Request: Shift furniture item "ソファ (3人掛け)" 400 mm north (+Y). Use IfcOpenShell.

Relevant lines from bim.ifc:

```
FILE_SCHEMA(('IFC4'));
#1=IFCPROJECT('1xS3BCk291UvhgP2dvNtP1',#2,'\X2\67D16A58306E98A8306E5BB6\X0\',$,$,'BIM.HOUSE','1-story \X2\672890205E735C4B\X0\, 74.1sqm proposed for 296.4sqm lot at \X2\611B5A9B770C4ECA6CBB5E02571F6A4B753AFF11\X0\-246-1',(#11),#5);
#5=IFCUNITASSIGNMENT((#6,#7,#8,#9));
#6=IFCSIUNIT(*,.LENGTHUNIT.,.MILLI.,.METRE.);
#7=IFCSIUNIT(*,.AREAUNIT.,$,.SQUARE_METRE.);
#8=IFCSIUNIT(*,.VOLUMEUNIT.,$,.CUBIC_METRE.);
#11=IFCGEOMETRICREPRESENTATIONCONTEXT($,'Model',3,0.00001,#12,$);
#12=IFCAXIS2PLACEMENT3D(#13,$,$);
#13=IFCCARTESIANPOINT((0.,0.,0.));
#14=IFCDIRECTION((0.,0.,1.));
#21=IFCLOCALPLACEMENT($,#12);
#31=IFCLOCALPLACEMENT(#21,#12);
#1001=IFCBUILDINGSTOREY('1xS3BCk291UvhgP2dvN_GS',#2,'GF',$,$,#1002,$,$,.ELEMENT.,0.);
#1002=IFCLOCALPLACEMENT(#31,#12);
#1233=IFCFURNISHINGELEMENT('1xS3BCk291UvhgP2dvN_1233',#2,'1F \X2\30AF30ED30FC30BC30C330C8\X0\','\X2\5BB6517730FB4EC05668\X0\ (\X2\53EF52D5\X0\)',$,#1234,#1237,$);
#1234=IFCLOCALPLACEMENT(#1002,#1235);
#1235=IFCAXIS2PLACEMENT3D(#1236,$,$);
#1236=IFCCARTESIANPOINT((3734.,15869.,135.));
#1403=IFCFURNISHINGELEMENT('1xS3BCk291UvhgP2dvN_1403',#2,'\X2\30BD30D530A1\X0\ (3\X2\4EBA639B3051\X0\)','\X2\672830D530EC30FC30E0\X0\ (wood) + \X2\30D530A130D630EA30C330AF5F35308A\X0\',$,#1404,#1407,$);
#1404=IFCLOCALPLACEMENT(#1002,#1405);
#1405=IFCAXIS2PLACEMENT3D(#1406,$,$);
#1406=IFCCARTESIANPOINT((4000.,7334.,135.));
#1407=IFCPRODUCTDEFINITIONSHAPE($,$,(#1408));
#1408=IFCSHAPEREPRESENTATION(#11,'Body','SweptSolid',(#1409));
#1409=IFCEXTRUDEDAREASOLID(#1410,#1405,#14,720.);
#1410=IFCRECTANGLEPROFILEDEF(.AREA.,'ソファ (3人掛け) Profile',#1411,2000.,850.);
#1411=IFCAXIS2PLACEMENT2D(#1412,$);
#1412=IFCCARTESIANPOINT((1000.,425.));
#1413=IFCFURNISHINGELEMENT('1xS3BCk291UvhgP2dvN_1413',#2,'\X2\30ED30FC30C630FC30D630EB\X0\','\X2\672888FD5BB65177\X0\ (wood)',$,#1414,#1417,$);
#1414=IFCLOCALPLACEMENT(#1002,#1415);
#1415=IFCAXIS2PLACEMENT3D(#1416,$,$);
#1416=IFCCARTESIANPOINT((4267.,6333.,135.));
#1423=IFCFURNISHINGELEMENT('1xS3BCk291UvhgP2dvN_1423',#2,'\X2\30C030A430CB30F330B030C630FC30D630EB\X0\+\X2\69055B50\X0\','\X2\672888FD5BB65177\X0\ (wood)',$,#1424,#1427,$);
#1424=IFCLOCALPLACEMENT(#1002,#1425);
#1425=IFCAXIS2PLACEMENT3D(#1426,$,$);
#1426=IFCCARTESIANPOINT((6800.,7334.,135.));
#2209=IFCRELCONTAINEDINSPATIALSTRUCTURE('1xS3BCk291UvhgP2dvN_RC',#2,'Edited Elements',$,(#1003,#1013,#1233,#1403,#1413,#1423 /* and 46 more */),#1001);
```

```python
import ifcopenshell
import ifcopenshell.api.geometry
import ifcopenshell.util.placement
import ifcopenshell.util.unit

model = ifcopenshell.open("bim.ifc")
unit_scale = ifcopenshell.util.unit.calculate_unit_scale(model)

item = model.by_guid("1xS3BCk291UvhgP2dvN_1403")
matrix = ifcopenshell.util.placement.get_local_placement(item.ObjectPlacement)
matrix[1, 3] += 0.4 / unit_scale
ifcopenshell.api.geometry.edit_object_placement(model, product=item, matrix=matrix, is_si=False)

print(ifcopenshell.util.placement.get_local_placement(item.ObjectPlacement).round(3) + 0.0)

model.write("bim_rev.ifc")
```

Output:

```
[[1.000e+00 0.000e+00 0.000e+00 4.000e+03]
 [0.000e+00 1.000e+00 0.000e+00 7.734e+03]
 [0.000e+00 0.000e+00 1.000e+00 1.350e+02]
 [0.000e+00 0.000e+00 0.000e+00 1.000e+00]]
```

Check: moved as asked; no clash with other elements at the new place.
